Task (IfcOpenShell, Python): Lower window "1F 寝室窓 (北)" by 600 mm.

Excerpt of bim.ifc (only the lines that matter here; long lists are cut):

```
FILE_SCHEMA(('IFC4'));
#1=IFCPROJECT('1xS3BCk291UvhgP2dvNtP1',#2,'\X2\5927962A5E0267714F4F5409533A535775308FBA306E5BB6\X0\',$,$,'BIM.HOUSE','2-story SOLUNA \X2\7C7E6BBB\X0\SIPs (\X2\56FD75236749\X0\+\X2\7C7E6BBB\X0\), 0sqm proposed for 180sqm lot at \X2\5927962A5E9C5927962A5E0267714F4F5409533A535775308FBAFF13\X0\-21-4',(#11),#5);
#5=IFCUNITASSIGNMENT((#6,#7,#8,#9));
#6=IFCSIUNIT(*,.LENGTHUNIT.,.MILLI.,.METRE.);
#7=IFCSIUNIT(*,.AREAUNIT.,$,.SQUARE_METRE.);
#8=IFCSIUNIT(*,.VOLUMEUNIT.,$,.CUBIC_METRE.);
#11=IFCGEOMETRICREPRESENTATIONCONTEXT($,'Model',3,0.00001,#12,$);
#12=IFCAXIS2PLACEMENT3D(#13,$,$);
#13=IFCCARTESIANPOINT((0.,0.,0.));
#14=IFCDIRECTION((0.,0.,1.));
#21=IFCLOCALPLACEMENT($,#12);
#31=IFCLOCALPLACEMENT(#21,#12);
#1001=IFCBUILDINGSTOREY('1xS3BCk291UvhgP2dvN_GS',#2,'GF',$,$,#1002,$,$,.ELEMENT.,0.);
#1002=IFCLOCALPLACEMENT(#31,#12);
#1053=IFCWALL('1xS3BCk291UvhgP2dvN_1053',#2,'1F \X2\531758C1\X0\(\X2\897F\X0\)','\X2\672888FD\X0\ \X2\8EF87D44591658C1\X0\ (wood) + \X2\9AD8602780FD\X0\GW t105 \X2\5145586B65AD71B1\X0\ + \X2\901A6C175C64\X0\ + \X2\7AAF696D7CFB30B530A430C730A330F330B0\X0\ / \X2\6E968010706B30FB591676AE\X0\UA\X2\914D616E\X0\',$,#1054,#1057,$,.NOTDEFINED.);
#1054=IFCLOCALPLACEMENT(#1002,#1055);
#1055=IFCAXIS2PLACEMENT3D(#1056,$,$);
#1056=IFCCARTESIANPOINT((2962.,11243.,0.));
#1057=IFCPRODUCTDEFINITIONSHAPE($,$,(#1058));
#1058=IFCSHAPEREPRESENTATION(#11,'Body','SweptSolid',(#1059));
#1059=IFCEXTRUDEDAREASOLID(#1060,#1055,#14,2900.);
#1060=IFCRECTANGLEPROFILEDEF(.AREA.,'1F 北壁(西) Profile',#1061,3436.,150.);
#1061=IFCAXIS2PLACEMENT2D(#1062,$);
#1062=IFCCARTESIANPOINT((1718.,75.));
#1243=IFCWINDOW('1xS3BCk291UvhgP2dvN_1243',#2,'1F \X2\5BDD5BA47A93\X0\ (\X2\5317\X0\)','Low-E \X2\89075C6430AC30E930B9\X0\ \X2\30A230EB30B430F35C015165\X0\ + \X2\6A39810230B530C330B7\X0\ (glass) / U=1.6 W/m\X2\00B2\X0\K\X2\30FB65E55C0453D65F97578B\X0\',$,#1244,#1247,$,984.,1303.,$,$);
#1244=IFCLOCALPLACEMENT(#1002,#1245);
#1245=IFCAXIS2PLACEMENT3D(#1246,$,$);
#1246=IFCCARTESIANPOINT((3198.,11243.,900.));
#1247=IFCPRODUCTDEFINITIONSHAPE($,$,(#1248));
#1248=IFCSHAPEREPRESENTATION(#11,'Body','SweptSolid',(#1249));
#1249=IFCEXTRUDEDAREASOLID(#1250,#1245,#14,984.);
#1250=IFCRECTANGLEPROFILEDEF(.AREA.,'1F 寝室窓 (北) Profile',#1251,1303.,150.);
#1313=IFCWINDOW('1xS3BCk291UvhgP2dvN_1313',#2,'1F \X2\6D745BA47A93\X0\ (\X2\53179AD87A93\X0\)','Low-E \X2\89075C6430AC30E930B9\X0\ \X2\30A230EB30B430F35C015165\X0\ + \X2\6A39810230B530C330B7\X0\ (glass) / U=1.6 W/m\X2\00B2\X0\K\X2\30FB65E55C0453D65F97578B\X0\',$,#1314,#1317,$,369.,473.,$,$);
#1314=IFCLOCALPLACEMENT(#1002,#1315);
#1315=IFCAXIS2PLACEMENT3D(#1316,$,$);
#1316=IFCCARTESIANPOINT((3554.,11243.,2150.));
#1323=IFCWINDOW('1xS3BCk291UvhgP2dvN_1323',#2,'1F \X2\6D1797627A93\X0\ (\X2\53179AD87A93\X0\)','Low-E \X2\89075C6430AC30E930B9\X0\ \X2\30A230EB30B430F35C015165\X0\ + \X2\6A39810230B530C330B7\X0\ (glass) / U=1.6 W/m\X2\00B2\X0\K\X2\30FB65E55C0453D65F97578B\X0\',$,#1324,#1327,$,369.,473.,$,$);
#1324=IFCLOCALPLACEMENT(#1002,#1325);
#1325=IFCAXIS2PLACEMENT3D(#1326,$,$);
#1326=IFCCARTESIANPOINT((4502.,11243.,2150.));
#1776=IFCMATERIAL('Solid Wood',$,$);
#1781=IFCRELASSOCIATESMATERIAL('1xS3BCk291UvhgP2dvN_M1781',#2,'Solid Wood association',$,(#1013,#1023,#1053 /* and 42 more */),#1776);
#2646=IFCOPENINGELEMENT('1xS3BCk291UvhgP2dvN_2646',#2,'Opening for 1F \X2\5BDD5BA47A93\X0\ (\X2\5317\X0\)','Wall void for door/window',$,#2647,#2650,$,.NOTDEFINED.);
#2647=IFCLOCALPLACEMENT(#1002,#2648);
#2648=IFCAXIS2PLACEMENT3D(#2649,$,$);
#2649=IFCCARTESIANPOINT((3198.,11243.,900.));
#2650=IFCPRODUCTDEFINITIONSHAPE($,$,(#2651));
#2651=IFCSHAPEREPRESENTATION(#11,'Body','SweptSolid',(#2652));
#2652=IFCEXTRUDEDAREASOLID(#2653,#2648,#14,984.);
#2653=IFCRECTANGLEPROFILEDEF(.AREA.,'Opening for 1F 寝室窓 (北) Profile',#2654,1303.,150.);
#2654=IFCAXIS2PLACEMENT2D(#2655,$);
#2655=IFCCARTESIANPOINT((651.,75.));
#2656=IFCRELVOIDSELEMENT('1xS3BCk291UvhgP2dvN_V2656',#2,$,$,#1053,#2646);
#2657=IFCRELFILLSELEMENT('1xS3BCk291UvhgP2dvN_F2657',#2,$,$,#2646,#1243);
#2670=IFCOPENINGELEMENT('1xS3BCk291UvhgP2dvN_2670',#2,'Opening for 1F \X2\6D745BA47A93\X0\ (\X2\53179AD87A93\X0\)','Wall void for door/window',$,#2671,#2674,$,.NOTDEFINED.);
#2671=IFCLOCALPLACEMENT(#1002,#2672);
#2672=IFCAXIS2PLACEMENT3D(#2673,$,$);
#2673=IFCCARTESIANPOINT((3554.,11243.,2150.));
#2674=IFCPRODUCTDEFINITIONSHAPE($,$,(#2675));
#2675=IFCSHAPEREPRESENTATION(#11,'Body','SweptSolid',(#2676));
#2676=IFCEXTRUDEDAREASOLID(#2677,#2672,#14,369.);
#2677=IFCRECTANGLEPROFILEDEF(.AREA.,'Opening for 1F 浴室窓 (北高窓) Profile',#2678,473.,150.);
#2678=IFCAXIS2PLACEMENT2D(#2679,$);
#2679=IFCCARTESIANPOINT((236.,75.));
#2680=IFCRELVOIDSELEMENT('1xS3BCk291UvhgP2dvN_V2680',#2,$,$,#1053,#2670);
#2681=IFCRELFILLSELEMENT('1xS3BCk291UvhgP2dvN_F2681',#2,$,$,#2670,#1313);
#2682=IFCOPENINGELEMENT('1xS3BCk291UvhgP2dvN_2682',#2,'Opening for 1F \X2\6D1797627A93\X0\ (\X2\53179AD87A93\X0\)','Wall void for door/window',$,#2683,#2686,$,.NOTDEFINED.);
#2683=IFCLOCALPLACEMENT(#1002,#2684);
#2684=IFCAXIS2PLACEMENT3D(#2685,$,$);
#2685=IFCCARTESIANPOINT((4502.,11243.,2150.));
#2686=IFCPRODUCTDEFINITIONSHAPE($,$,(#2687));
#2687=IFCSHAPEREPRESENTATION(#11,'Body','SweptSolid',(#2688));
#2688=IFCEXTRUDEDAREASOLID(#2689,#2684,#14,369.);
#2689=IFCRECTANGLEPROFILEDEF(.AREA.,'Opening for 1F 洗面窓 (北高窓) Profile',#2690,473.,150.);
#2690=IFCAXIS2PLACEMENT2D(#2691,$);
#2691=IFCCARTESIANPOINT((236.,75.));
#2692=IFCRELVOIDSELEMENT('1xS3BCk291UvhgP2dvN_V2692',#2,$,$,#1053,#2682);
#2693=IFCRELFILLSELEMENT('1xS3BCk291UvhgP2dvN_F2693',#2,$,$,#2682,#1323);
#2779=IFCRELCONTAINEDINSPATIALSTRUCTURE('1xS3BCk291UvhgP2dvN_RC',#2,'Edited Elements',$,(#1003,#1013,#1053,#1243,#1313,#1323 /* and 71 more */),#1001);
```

```python
import numpy as np
import ifcopenshell
import ifcopenshell.api.geometry
import ifcopenshell.util.placement
import ifcopenshell.util.unit

model = ifcopenshell.open("bim.ifc")
unit_scale = ifcopenshell.util.unit.calculate_unit_scale(model)

window = model.by_id(1243)
opening = window.FillsVoids[0].RelatingOpeningElement
dz = -0.6 / unit_scale

shift = np.array([0.0, 0.0, dz])
# The window is not placed relative to its opening, so move both.
for product in (opening, window):
    matrix = ifcopenshell.util.placement.get_local_placement(product.ObjectPlacement)
    matrix[:3, 3] += shift
    ifcopenshell.api.geometry.edit_object_placement(model, product=product, matrix=matrix, is_si=False)

print(f"moved by {dz * unit_scale:+.3f} m")

model.write("bim_edited.ifc")
```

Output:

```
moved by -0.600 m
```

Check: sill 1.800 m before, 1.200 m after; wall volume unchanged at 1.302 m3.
